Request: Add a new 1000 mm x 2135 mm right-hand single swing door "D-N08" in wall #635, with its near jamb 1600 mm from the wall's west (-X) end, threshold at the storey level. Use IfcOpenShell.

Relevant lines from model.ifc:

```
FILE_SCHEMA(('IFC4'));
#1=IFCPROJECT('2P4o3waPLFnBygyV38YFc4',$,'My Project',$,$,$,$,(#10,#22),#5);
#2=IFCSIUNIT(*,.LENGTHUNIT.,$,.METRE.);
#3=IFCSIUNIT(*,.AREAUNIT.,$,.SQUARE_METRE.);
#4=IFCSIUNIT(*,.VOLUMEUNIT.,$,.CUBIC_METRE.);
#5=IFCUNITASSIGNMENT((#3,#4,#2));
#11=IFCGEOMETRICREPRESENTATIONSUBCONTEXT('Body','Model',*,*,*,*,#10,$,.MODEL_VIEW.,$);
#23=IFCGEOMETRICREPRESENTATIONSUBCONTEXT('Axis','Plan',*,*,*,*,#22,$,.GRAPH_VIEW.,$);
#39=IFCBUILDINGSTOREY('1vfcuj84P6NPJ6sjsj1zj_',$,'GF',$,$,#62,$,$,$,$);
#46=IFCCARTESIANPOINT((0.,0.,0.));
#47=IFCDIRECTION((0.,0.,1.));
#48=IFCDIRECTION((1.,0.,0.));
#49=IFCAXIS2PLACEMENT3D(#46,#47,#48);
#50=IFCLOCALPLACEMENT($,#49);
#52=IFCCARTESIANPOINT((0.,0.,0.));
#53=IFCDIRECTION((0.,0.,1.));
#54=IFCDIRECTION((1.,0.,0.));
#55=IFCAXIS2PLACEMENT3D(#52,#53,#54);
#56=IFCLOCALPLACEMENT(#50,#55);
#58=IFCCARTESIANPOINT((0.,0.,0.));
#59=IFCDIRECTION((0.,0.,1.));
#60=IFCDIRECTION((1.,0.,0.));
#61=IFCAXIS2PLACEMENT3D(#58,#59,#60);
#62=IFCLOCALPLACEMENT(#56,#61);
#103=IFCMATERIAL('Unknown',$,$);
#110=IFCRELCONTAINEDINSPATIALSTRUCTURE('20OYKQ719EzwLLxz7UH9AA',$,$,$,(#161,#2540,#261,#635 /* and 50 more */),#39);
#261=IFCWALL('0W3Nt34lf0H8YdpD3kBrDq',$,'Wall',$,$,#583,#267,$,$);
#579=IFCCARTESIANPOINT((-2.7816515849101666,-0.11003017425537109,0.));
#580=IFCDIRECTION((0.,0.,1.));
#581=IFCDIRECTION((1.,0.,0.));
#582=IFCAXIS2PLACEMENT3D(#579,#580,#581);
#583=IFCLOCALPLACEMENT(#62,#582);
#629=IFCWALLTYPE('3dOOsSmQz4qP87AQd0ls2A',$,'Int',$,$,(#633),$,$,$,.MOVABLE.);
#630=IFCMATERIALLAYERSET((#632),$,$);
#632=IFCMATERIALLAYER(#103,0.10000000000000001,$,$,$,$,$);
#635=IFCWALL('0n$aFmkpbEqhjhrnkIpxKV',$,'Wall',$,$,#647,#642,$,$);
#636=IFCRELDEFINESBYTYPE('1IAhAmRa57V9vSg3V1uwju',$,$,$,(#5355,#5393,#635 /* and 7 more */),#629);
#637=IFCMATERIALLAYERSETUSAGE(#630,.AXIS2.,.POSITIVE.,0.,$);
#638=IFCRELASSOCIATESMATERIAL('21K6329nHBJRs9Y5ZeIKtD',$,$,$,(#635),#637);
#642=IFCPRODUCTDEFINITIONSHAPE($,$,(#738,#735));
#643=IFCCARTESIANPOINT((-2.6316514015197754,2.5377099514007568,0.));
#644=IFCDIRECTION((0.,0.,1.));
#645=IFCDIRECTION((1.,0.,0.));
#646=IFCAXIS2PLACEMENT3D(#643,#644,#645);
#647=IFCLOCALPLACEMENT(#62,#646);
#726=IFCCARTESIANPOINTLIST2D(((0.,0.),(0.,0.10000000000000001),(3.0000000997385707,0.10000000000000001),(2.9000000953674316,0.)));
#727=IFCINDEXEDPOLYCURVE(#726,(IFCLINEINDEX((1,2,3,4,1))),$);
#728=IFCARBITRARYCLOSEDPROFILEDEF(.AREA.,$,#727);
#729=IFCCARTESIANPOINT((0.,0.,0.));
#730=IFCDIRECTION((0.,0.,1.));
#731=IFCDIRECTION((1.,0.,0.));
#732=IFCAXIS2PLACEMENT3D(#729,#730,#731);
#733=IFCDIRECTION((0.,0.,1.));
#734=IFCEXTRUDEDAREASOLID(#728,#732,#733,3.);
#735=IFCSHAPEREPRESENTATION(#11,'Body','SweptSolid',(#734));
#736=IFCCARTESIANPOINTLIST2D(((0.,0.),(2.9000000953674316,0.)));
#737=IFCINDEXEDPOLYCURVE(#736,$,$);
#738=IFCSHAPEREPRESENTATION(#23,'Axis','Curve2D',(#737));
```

```python
import numpy as np
import ifcopenshell
import ifcopenshell.api.feature
import ifcopenshell.api.geometry
import ifcopenshell.api.root
import ifcopenshell.api.spatial
import ifcopenshell.geom
import ifcopenshell.util.element
import ifcopenshell.util.placement
import ifcopenshell.util.representation
import ifcopenshell.util.shape
import ifcopenshell.util.unit

model = ifcopenshell.open("model.ifc")
unit_scale = ifcopenshell.util.unit.calculate_unit_scale(model)
settings = ifcopenshell.geom.settings()


def volume(element):
    """Net volume in cubic metres, openings subtracted."""
    shape = ifcopenshell.geom.create_shape(settings, element)
    return ifcopenshell.util.shape.get_volume(shape.geometry)


wall = model.by_id(635)
storey = ifcopenshell.util.element.get_container(wall, ifc_class="IfcBuildingStorey")
context = ifcopenshell.util.representation.get_context(model, "Model", "Body", "MODEL_VIEW")
before = volume(wall)

width, height, from_end, sill = 1, 2.135, 1.6, 0.0  # metres

# The wall runs along its own X axis, and the end named is its -X end.
wall_shape = ifcopenshell.geom.create_shape(settings, wall)
x, y, z = ifcopenshell.util.shape.get_vertices(wall_shape.geometry).T
start = x.min() + from_end
face, thickness = float(y.min()), float(y.max() - y.min())
wall_matrix = ifcopenshell.util.placement.get_local_placement(wall.ObjectPlacement)
level = ifcopenshell.util.placement.get_local_placement(storey.ObjectPlacement)[2, 3]


def in_wall(x, y):
    """Placement at x, y metres in the wall's axes, at sill height."""
    matrix = wall_matrix.copy()
    matrix[:, 3] = wall_matrix @ np.array([x / unit_scale, y / unit_scale, 0.0, 1.0])
    matrix[2, 3] = level + sill / unit_scale
    return matrix


# Opening: a box that overshoots both wall faces by 50 mm.
opening = ifcopenshell.api.root.create_entity(model, ifc_class="IfcOpeningElement", predefined_type="OPENING")
box = ifcopenshell.api.geometry.add_wall_representation(
    model, context=context, length=width, height=height, thickness=thickness + 0.1
)
ifcopenshell.api.geometry.assign_representation(model, product=opening, representation=box)
ifcopenshell.api.geometry.edit_object_placement(model, product=opening, matrix=in_wall(start, face - 0.05), is_si=False)
ifcopenshell.api.feature.add_feature(model, feature=opening, element=wall)

door = ifcopenshell.api.root.create_entity(model, ifc_class="IfcDoor", name="D-N08", predefined_type="DOOR")
door.OverallWidth, door.OverallHeight = width / unit_scale, height / unit_scale
door.OperationType = "SINGLE_SWING_RIGHT"
body = ifcopenshell.api.geometry.add_door_representation(
    model,
    context=context,
    overall_width=door.OverallWidth,
    overall_height=door.OverallHeight,
    operation_type="SINGLE_SWING_RIGHT",
    lining_properties={"LiningDepth": thickness / unit_scale, "ThresholdDepth": thickness / unit_scale},
)
ifcopenshell.api.geometry.assign_representation(model, product=door, representation=body)
ifcopenshell.api.spatial.assign_container(model, products=[door], relating_structure=storey)
ifcopenshell.api.feature.add_filling(model, opening=opening, element=door)

# The lining spans the wall, so the door starts at the wall face.
ifcopenshell.api.geometry.edit_object_placement(model, product=door, matrix=in_wall(start, face), is_si=False)

after = volume(wall)

print(f"wall volume {before:.3f} -> {after:.3f} m3")

model.write("model-out.ifc")
```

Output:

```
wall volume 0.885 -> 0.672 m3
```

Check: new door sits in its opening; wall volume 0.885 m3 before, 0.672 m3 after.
